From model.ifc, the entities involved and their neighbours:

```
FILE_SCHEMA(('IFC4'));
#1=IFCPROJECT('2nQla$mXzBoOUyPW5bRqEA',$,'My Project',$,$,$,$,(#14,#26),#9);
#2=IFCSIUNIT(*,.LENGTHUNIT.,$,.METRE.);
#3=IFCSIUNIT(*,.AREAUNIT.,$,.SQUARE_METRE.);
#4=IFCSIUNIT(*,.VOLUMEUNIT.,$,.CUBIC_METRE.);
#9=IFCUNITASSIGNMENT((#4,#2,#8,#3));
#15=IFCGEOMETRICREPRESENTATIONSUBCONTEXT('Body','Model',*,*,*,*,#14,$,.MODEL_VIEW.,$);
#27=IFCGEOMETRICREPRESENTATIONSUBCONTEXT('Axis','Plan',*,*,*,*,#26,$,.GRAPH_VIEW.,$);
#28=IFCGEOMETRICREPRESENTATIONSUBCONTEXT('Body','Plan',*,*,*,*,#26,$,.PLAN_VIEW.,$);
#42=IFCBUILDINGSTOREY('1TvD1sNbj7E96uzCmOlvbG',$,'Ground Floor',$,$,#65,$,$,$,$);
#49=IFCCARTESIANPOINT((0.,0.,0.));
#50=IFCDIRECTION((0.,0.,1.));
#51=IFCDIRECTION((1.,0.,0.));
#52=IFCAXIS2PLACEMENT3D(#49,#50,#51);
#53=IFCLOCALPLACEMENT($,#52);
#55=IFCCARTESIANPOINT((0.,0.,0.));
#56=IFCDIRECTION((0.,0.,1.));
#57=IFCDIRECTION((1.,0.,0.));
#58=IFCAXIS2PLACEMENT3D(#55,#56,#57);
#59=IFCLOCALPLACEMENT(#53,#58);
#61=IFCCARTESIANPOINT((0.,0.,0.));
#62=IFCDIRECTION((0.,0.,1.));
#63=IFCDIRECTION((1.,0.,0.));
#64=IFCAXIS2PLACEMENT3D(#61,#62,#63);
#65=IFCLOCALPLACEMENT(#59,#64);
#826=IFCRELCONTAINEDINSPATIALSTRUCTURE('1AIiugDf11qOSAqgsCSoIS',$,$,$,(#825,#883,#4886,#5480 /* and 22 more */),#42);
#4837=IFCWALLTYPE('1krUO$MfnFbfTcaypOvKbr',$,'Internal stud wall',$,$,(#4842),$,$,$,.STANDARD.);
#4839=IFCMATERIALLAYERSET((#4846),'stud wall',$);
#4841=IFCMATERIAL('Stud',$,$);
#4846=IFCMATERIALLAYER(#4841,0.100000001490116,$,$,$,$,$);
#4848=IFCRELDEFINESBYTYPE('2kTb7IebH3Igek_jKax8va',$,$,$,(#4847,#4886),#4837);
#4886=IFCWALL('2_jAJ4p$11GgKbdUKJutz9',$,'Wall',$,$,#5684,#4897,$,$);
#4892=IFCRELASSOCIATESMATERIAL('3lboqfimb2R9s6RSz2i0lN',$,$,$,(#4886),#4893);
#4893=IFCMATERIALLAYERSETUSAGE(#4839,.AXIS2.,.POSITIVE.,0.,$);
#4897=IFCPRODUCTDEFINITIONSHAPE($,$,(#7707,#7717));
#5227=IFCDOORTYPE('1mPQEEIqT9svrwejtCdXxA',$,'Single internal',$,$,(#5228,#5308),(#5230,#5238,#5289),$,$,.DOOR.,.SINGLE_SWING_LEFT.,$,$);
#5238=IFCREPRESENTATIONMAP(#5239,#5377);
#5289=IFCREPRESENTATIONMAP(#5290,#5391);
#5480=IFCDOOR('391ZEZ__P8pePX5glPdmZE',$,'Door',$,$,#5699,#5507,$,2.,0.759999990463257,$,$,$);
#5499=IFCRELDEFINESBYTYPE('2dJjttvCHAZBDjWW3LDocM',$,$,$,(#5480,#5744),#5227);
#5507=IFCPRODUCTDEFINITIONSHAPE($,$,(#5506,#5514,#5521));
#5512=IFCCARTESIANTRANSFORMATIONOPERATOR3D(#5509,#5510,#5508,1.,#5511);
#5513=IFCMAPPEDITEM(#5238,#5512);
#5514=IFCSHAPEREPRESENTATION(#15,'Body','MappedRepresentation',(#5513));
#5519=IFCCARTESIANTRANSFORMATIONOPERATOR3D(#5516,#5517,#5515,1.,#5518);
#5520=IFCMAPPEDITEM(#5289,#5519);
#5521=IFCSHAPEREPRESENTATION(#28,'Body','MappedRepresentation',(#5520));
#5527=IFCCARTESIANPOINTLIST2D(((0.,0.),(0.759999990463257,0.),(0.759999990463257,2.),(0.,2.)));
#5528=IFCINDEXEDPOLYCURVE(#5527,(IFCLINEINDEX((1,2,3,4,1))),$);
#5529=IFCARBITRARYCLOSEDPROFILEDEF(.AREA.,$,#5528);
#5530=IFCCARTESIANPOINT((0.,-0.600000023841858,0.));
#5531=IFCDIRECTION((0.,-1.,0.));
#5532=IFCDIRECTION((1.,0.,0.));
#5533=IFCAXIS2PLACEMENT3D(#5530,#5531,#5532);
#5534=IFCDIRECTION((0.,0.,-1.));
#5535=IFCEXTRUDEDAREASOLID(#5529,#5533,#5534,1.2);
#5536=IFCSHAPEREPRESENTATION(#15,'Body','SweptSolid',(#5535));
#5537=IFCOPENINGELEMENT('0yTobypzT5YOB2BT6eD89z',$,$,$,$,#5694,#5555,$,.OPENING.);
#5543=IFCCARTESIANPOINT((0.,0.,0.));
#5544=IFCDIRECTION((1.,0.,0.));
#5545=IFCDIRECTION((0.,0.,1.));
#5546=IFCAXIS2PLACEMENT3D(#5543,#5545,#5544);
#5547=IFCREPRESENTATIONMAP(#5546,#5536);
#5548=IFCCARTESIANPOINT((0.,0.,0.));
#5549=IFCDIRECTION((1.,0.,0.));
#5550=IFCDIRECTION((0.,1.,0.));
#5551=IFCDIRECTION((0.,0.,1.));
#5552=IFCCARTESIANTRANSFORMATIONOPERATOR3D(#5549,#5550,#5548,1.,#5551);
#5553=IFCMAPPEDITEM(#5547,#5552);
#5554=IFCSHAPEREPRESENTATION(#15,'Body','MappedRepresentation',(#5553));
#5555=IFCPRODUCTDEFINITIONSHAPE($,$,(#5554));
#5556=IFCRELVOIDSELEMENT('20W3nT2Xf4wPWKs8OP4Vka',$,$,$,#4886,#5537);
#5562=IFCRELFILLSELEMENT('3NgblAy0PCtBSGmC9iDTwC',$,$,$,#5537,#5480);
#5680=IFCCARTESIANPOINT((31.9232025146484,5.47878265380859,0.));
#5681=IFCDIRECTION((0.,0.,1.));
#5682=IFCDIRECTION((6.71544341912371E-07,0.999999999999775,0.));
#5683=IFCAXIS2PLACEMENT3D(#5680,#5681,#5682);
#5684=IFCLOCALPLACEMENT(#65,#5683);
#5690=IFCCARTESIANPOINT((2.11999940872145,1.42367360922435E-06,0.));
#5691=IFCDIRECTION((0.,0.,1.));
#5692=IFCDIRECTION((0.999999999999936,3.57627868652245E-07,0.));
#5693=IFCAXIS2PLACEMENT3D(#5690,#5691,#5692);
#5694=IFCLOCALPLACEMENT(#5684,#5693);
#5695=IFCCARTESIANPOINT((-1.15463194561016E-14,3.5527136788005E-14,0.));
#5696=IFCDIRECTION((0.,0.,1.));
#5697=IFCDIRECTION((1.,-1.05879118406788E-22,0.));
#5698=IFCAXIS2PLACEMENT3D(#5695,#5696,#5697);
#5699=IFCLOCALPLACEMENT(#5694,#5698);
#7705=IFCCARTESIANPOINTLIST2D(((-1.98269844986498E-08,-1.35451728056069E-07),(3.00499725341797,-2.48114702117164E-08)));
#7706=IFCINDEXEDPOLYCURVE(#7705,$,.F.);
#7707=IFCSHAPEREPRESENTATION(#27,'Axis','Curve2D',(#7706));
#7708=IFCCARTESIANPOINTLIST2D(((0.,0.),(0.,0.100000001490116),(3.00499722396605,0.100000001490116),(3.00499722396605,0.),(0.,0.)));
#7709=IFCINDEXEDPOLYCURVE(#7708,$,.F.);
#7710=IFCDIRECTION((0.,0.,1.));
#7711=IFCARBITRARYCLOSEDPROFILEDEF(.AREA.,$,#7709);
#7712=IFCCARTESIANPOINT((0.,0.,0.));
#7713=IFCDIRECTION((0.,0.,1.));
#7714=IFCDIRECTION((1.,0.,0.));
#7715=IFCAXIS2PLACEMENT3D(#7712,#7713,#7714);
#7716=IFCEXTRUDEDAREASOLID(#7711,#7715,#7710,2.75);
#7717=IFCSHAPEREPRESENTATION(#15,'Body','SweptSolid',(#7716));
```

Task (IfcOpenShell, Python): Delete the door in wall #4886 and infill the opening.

```python
import ifcopenshell
import ifcopenshell.api.feature
import ifcopenshell.api.root
import ifcopenshell.geom
import ifcopenshell.util.shape

model = ifcopenshell.open("model.ifc")
settings = ifcopenshell.geom.settings()


def volume(element):
    """Net volume in cubic metres, openings subtracted."""
    shape = ifcopenshell.geom.create_shape(settings, element)
    return ifcopenshell.util.shape.get_volume(shape.geometry)


door = model.by_guid("391ZEZ__P8pePX5glPdmZE")
opening = door.FillsVoids[0].RelatingOpeningElement
wall = opening.VoidsElements[0].RelatingBuildingElement
before = volume(wall)

ifcopenshell.api.root.remove_product(model, product=door)
ifcopenshell.api.feature.remove_feature(model, feature=opening)

after = volume(wall)

print(f"wall volume {before:.3f} -> {after:.3f} m3")

model.write("model_rev.ifc")
```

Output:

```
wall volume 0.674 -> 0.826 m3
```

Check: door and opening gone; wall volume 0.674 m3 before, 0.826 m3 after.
